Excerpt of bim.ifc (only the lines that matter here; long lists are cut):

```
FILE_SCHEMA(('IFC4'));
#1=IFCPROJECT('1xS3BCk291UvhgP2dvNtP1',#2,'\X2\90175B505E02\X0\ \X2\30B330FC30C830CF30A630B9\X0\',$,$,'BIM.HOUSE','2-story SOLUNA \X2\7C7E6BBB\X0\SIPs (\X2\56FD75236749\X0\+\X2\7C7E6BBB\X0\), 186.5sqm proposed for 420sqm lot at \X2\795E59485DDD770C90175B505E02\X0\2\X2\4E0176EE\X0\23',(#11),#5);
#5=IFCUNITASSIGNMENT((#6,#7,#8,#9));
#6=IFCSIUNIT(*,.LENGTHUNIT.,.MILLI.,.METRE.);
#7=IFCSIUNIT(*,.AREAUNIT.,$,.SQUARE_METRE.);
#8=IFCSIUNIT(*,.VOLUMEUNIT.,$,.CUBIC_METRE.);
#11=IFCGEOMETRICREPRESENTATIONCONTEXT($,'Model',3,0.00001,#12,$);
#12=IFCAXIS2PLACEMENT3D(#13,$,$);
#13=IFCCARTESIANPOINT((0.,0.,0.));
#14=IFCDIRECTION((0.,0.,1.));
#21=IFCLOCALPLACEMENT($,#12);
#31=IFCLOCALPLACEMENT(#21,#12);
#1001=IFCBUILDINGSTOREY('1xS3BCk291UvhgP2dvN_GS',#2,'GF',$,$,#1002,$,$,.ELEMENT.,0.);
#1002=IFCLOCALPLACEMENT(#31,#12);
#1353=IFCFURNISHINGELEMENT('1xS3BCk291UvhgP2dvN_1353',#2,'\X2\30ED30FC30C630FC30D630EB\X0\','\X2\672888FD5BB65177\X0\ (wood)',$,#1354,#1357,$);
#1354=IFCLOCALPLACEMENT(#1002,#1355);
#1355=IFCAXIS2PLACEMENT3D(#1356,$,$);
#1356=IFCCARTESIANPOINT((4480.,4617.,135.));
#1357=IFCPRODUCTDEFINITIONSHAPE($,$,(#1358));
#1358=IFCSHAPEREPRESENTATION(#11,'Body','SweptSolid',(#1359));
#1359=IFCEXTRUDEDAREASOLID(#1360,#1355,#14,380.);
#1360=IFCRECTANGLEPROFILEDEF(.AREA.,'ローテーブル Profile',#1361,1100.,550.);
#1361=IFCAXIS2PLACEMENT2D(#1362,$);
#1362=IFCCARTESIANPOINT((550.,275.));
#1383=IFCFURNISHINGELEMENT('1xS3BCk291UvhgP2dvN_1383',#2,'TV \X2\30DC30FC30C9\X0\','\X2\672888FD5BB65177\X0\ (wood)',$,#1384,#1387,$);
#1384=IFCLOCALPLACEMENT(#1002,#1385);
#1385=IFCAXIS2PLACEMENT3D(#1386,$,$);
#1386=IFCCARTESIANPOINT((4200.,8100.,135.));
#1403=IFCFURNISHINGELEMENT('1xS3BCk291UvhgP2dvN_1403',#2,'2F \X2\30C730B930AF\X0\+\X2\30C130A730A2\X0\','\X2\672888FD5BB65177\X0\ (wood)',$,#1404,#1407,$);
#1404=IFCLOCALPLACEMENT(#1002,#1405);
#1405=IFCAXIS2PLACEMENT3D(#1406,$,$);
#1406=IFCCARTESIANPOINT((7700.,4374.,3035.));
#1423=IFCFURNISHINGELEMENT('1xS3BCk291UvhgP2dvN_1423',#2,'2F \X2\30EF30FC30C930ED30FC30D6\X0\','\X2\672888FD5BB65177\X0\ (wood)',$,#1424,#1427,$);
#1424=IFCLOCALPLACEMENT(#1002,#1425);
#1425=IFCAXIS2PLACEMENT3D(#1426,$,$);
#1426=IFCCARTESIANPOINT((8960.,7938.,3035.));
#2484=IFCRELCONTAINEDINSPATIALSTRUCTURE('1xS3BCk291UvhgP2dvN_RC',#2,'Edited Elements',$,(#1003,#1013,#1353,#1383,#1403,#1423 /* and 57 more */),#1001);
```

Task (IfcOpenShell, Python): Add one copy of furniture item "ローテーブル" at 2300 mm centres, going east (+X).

```python
import numpy as np
import ifcopenshell
import ifcopenshell.api.geometry
import ifcopenshell.api.root
import ifcopenshell.util.element
import ifcopenshell.util.placement
import ifcopenshell.util.unit

model = ifcopenshell.open("bim.ifc")
unit_scale = ifcopenshell.util.unit.calculate_unit_scale(model)


def reuse_history(source, copy):
    """copy_class also copies each property set's owner history, people and application; keep the originals."""
    for rel in copy.IsDefinedBy:
        if rel.is_a("IfcRelDefinesByProperties") and (history := rel.RelatingPropertyDefinition.OwnerHistory):
            rel.RelatingPropertyDefinition.OwnerHistory = source.OwnerHistory
            ifcopenshell.util.element.remove_deep2(model, history)


source = model.by_guid("1xS3BCk291UvhgP2dvN_1353")
base = ifcopenshell.util.placement.get_local_placement(source.ObjectPlacement)
step = np.array([1.0, 0.0, 0.0]) * 2.3 / unit_scale

for i in range(1, 2):
    copy = ifcopenshell.api.root.copy_class(model, product=source)
    copy.Representation = ifcopenshell.util.element.copy_deep(
        model, source.Representation, exclude=["IfcGeometricRepresentationContext", "IfcRepresentationMap"]
    )
    reuse_history(source, copy)
    matrix = base.copy()
    matrix[:3, 3] += i * step
    print("added at", matrix[:3, 3].round(3) + 0.0)
    ifcopenshell.api.geometry.edit_object_placement(model, product=copy, matrix=matrix, is_si=False)

model.write("bim_rev.ifc")
```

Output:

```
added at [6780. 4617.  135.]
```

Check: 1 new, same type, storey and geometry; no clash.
